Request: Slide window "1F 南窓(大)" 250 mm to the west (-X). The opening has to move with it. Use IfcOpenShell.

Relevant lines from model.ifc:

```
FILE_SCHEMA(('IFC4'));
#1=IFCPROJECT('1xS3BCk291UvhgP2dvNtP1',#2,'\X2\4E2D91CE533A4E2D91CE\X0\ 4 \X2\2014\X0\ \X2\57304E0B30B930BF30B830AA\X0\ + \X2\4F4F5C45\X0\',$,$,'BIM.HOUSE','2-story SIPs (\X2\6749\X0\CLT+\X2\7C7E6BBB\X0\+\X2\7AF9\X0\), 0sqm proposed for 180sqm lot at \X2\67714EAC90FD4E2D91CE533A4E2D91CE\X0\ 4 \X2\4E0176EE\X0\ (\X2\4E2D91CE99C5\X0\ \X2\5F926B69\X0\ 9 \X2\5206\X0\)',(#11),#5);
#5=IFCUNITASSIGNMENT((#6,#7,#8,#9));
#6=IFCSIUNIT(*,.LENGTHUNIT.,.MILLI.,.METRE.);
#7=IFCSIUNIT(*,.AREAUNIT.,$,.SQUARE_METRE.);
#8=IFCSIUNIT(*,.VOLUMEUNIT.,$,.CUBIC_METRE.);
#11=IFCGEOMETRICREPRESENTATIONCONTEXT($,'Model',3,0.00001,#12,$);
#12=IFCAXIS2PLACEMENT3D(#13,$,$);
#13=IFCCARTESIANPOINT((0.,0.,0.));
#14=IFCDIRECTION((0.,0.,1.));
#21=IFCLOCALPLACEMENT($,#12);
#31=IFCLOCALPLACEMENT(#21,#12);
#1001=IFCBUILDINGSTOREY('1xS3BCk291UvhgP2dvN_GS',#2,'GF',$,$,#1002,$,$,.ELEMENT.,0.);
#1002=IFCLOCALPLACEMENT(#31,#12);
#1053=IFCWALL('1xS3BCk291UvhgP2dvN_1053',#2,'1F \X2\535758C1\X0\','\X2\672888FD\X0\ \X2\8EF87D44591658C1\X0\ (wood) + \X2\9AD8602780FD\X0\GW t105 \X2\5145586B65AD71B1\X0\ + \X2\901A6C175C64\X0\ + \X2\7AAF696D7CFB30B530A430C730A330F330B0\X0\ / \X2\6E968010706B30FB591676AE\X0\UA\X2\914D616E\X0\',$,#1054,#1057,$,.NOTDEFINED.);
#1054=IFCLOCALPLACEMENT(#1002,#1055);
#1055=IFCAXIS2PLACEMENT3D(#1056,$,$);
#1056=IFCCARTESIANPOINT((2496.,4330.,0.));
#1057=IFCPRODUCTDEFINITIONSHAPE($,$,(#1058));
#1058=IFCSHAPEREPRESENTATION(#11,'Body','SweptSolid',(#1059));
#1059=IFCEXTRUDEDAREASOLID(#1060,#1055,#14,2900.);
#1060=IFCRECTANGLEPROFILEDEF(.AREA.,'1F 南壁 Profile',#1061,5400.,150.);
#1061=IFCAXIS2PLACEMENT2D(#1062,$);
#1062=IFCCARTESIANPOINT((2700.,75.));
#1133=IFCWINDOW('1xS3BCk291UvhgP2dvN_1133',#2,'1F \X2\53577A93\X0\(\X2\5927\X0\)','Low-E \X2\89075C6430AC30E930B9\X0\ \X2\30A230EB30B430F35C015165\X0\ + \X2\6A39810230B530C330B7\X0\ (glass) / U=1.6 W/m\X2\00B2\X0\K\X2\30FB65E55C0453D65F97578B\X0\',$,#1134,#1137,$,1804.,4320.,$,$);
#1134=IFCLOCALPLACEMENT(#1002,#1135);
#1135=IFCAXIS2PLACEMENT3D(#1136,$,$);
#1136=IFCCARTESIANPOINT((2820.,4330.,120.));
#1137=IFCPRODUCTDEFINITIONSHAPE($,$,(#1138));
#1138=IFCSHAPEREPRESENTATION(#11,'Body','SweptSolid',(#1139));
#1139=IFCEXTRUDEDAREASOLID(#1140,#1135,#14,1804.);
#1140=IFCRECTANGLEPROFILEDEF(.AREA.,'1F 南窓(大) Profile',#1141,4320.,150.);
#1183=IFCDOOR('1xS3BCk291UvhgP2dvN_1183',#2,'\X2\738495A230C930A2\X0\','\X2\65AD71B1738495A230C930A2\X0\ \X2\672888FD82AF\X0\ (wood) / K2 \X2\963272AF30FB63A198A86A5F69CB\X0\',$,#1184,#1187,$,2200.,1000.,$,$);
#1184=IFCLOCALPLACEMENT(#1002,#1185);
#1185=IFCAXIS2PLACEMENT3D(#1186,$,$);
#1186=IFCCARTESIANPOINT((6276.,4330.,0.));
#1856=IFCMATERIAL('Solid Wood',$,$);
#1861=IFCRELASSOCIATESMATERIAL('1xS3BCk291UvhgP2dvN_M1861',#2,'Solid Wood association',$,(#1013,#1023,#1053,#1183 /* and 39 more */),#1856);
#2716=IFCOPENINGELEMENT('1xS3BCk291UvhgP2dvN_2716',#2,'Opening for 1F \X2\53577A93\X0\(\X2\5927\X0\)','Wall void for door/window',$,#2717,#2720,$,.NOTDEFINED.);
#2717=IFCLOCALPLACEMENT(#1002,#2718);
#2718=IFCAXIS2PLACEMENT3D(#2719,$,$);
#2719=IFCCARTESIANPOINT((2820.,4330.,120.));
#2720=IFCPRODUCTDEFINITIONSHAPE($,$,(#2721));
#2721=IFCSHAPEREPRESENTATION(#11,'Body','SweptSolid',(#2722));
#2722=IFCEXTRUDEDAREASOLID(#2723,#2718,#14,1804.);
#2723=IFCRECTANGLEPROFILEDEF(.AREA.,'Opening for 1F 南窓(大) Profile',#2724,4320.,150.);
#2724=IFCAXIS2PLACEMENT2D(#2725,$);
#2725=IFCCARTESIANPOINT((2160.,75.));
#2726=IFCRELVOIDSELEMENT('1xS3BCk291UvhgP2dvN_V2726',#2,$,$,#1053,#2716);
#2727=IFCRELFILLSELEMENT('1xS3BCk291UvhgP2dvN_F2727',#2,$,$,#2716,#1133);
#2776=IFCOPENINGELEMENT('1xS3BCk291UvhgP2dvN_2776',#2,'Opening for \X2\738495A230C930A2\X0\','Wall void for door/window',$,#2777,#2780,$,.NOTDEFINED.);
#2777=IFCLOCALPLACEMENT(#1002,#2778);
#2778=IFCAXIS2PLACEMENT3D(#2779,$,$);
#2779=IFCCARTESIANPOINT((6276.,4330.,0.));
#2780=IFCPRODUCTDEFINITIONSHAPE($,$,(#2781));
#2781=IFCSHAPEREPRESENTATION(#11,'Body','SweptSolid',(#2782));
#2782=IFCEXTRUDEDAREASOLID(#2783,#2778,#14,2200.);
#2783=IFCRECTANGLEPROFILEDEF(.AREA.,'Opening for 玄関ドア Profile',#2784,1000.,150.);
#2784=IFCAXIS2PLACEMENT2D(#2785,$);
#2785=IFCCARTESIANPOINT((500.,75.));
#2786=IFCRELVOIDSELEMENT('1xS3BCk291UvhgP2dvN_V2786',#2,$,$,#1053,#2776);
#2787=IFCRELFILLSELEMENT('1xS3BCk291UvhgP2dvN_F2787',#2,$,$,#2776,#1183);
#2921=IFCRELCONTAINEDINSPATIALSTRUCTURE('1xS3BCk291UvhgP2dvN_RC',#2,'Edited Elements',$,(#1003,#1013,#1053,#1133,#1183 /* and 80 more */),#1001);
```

```python
import ifcopenshell
import ifcopenshell.api.geometry
import ifcopenshell.util.placement
import ifcopenshell.util.unit

model = ifcopenshell.open("model.ifc")
unit_scale = ifcopenshell.util.unit.calculate_unit_scale(model)

window = model.by_guid("1xS3BCk291UvhgP2dvN_1133")
opening = window.FillsVoids[0].RelatingOpeningElement
wall = opening.VoidsElements[0].RelatingBuildingElement

wall_matrix = ifcopenshell.util.placement.get_local_placement(wall.ObjectPlacement)
shift = wall_matrix[:3, 0] * -0.25 / unit_scale
before = ifcopenshell.util.placement.get_local_placement(window.ObjectPlacement)[:3, 3].copy()

# The window is not placed relative to its opening, so move both.
for product in (opening, window):
    matrix = ifcopenshell.util.placement.get_local_placement(product.ObjectPlacement)
    matrix[:3, 3] += shift
    ifcopenshell.api.geometry.edit_object_placement(model, product=product, matrix=matrix, is_si=False)

after = ifcopenshell.util.placement.get_local_placement(window.ObjectPlacement)[:3, 3]
print("window moved by", (after - before).round(3) + 0.0)

model.write("model_v2.ifc")
```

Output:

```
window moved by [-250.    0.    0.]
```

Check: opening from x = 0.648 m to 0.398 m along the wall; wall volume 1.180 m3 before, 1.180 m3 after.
